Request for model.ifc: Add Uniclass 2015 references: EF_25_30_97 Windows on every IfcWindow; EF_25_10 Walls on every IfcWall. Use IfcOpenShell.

First a look at what the model holds.

```python
import ifcopenshell

model = ifcopenshell.open("model.ifc")
print(model.schema)
print("classifications:", [c.Name for c in model.by_type("IfcClassification")])
for ifc_class in ("IfcDoor", "IfcRoof", "IfcStair", "IfcWall", "IfcWindow"):
    print(ifc_class, len(model.by_type(ifc_class)))
```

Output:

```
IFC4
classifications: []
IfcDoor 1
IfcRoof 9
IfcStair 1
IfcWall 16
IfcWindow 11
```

```python
import ifcopenshell
import ifcopenshell.api.classification

model = ifcopenshell.open("model.ifc")

system = ifcopenshell.api.classification.add_classification(model, classification="Uniclass 2015")

codes = {
    "IfcWindow": ("EF_25_30_97", "Windows"),
    "IfcWall": ("EF_25_10", "Walls"),
}
for ifc_class, (code, name) in codes.items():
    products = model.by_type(ifc_class)
    ifcopenshell.api.classification.add_reference(
        model, products=products, classification=system, identification=code, name=name
    )
    print(code, len(products))

model.write("model_edited.ifc")
```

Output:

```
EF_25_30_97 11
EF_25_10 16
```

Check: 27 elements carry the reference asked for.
